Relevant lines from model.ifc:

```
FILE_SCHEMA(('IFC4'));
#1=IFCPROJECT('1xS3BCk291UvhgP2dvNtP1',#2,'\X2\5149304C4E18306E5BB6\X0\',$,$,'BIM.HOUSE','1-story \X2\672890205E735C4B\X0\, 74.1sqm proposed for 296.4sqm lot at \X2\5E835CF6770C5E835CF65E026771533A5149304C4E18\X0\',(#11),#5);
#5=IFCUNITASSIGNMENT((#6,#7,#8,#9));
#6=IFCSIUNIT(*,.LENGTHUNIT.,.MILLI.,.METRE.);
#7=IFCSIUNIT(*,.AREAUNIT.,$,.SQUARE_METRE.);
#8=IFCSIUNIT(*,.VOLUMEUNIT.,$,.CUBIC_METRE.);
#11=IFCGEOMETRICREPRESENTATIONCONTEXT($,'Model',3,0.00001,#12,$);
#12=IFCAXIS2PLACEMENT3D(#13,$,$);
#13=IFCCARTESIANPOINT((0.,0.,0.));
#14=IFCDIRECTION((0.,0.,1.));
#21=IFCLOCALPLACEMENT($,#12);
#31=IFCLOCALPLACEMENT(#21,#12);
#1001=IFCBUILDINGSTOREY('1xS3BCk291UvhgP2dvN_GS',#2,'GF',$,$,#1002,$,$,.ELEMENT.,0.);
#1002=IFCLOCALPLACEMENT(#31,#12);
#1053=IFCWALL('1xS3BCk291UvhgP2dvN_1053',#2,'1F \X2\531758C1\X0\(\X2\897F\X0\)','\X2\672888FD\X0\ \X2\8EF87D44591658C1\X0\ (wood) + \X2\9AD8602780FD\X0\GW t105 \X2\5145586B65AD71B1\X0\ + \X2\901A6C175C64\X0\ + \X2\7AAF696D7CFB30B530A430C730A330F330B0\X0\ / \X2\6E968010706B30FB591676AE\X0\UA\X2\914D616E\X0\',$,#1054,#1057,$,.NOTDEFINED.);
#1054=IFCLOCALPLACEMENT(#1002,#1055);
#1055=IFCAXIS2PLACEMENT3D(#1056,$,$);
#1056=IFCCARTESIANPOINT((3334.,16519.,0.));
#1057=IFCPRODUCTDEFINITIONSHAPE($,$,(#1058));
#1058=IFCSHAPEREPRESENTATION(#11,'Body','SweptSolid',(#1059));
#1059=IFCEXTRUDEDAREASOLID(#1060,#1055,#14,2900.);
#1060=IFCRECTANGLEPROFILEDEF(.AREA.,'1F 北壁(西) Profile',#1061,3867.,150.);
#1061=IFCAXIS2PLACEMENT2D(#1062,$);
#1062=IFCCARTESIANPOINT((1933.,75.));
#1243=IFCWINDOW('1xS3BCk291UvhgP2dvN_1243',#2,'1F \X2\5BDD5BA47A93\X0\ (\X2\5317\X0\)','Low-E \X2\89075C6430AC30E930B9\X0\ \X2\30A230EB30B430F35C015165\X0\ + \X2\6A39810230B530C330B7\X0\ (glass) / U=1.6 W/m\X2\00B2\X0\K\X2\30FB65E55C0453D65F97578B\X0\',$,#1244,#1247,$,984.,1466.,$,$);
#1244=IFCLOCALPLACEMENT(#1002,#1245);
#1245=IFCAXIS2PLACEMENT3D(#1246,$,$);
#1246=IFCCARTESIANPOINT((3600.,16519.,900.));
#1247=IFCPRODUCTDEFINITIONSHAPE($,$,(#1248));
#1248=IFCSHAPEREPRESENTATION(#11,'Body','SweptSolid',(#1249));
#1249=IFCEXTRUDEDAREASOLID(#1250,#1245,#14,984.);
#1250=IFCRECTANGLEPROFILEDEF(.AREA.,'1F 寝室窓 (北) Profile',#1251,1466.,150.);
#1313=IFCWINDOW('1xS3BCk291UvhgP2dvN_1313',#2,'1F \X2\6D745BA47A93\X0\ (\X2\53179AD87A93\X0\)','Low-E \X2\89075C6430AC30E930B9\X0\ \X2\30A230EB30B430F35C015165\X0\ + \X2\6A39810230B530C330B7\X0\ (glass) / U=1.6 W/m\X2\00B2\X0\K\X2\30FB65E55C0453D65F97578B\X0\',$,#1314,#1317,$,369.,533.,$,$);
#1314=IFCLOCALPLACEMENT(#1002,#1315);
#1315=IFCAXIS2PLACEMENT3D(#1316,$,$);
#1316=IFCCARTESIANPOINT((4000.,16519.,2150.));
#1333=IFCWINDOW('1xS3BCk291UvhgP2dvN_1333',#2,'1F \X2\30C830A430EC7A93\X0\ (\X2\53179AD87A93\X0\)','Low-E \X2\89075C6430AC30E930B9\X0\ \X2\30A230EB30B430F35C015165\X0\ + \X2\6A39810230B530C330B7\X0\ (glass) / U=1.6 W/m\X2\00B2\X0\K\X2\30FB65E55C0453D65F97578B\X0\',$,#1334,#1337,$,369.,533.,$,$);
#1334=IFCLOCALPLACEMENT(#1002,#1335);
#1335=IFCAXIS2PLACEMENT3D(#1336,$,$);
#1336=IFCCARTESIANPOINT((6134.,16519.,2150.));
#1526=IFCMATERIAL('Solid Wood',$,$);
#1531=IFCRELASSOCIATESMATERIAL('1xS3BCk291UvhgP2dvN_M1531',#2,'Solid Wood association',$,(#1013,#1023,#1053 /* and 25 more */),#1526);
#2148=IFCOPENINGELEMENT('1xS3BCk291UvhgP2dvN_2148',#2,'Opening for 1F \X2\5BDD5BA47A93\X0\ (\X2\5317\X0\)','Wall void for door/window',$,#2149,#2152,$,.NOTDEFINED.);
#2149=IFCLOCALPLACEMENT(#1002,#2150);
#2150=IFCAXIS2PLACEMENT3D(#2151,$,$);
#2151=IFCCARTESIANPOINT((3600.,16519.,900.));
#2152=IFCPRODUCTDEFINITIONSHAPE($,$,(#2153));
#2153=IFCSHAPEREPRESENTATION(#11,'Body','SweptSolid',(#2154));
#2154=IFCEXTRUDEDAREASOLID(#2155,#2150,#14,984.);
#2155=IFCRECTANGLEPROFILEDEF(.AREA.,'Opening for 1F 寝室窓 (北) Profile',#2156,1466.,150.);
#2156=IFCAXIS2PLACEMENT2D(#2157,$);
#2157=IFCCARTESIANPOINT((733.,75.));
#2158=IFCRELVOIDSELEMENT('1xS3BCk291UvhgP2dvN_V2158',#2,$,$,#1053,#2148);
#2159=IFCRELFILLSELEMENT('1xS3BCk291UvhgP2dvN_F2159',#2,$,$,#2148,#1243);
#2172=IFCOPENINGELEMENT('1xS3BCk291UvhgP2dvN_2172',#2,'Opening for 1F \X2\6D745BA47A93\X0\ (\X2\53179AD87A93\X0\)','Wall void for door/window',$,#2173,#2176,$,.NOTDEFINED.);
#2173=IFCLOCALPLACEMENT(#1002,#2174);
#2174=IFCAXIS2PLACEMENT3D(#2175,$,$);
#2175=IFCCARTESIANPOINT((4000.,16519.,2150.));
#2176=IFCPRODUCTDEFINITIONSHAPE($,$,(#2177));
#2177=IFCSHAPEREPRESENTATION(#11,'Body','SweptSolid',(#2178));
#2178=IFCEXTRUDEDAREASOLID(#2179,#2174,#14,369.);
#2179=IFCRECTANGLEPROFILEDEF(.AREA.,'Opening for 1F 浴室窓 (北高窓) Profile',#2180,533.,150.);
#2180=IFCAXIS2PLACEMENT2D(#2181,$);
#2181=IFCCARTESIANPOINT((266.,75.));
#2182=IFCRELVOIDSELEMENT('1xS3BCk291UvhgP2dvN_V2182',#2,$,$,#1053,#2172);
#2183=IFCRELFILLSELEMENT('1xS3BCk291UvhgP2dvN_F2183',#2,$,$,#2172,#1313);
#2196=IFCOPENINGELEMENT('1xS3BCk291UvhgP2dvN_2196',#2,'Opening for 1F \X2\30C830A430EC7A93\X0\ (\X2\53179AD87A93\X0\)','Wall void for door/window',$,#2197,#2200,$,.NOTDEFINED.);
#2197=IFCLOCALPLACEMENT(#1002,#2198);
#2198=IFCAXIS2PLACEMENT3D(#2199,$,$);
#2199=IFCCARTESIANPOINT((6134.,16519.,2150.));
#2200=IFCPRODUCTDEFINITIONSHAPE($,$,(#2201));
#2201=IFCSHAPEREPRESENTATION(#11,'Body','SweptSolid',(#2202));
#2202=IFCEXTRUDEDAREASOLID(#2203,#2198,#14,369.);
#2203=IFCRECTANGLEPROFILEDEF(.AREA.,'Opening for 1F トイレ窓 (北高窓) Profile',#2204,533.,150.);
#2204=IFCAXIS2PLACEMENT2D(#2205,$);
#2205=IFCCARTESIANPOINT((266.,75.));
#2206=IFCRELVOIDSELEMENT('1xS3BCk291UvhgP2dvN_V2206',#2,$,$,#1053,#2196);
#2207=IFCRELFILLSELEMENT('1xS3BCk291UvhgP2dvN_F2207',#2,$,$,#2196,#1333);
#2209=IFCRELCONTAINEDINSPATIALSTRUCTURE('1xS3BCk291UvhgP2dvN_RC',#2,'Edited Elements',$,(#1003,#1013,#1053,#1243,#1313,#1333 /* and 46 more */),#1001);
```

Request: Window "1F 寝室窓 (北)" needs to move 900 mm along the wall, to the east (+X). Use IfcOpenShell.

```python
import ifcopenshell
import ifcopenshell.api.geometry
import ifcopenshell.util.placement

model = ifcopenshell.open("model.ifc")

window = model.by_guid("1xS3BCk291UvhgP2dvN_1243")
opening = window.FillsVoids[0].RelatingOpeningElement
wall = opening.VoidsElements[0].RelatingBuildingElement

wall_matrix = ifcopenshell.util.placement.get_local_placement(wall.ObjectPlacement)
shift = wall_matrix[:3, 0] * 900.0
before = ifcopenshell.util.placement.get_local_placement(window.ObjectPlacement)[:3, 3].copy()

# The window is not placed relative to its opening, so move both.
for product in (opening, window):
    matrix = ifcopenshell.util.placement.get_local_placement(product.ObjectPlacement)
    matrix[:3, 3] += shift
    ifcopenshell.api.geometry.edit_object_placement(model, product=product, matrix=matrix, is_si=False)

after = ifcopenshell.util.placement.get_local_placement(window.ObjectPlacement)[:3, 3]
print("window moved by", (after - before).round(3) + 0.0)

model.write("model_rev.ifc")
```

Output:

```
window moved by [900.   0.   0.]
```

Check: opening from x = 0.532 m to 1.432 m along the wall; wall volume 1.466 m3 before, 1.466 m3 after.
